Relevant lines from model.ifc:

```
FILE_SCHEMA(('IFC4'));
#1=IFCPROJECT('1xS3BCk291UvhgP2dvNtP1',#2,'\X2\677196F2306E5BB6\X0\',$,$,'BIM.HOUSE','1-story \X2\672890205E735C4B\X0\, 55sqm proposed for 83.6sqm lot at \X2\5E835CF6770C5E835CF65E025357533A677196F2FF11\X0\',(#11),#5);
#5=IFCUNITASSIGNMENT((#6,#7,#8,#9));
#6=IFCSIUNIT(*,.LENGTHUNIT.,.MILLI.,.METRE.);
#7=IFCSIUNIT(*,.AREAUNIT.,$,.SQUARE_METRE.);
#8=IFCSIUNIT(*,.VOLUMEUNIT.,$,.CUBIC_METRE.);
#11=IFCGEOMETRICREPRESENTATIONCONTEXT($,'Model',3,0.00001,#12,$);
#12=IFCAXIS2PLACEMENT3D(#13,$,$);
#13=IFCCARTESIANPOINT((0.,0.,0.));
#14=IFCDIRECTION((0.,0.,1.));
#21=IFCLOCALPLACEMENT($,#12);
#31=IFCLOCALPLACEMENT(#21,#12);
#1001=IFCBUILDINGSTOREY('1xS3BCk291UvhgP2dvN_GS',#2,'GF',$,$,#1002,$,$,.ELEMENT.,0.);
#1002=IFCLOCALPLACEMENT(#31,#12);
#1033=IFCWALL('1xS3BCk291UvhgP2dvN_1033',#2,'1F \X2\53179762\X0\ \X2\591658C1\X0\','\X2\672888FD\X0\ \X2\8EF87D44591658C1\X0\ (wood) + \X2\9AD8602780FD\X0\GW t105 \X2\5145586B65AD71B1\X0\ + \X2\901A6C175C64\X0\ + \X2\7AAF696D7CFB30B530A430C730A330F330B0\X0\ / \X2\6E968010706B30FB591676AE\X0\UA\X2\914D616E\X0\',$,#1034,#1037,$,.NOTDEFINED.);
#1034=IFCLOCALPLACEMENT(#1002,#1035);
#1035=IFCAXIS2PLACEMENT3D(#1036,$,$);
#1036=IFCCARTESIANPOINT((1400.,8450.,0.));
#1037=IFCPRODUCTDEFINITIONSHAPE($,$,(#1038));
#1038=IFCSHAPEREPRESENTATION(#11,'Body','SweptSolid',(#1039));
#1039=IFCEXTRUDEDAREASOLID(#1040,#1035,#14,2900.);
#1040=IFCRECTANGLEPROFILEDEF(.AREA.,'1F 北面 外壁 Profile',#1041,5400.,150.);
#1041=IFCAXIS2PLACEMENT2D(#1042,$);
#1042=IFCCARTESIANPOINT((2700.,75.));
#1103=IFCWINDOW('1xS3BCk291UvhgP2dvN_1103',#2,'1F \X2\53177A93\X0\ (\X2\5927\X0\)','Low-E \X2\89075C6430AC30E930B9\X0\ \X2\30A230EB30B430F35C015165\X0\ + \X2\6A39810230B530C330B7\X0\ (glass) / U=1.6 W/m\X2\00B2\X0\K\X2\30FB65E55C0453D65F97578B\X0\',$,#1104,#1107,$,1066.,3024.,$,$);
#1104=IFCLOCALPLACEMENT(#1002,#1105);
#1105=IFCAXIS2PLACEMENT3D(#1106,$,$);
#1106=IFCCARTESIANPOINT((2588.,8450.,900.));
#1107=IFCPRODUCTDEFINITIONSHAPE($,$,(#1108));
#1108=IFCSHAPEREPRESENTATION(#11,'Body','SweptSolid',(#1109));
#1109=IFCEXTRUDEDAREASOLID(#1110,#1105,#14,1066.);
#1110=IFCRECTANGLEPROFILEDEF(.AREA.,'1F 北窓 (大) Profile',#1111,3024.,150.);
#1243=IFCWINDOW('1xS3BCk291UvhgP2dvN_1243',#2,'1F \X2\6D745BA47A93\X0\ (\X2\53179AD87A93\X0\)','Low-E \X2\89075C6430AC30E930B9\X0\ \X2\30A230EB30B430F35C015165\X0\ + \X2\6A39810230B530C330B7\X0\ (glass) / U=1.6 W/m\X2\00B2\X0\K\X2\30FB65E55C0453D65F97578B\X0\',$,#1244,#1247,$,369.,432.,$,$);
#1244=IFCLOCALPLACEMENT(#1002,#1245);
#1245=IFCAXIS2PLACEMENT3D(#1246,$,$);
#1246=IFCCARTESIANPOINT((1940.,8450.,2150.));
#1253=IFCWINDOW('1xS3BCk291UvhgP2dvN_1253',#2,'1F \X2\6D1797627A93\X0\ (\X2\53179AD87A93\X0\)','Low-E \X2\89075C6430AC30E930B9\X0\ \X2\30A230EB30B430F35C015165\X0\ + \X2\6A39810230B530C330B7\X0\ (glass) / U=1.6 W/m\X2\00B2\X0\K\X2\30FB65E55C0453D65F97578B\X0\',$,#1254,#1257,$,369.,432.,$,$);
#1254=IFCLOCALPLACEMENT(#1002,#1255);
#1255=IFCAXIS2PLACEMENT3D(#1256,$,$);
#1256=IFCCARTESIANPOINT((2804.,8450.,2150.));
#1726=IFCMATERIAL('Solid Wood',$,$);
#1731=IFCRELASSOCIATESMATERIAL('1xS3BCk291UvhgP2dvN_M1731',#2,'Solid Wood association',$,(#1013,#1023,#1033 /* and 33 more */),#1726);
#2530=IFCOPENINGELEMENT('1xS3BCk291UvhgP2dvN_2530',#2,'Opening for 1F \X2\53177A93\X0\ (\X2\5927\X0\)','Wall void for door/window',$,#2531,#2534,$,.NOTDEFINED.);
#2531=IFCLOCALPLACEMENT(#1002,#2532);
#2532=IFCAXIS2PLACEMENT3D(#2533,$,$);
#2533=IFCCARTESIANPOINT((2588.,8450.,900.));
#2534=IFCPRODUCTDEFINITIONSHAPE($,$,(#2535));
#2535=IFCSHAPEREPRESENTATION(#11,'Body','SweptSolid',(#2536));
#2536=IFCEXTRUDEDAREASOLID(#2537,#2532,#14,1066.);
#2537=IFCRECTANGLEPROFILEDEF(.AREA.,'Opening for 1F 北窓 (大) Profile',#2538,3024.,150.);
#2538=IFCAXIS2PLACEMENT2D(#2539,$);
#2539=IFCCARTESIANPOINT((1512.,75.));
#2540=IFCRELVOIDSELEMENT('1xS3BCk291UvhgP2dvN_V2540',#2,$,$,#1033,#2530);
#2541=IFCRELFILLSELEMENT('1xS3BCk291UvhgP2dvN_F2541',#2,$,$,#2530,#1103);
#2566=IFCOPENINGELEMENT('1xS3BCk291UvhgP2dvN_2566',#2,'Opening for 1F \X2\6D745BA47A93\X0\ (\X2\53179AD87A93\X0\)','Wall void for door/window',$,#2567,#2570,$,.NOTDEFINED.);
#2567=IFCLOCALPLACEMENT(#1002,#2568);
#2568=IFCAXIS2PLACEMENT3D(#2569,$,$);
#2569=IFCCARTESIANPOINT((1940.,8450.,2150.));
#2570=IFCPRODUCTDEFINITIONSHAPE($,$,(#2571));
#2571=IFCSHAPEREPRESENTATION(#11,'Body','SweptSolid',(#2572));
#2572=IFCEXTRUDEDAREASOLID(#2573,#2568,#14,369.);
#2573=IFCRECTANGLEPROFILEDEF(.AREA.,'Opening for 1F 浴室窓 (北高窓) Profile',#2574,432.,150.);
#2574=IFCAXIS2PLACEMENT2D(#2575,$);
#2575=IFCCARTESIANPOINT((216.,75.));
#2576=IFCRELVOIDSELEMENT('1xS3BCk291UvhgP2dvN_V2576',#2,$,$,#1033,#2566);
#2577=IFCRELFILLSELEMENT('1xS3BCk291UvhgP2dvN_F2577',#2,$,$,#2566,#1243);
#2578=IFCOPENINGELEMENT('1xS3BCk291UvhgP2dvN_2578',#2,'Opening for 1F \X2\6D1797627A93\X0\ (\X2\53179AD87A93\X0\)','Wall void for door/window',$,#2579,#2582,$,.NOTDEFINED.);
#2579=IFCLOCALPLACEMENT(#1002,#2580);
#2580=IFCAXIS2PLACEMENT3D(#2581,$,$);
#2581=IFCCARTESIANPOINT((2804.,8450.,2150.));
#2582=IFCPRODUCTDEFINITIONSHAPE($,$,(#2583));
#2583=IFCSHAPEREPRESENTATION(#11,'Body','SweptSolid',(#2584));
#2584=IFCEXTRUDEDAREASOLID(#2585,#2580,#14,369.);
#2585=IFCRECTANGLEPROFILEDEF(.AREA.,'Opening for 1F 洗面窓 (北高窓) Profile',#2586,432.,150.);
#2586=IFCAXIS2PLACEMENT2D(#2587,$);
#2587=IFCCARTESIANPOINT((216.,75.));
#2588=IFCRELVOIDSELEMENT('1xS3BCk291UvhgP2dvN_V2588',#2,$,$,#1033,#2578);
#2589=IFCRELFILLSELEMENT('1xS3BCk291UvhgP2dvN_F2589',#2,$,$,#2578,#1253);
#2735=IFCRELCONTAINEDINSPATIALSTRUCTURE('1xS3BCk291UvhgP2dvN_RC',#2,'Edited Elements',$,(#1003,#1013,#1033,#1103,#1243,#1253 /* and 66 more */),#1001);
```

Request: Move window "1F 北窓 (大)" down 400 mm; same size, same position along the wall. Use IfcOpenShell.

```python
import numpy as np
import ifcopenshell
import ifcopenshell.api.geometry
import ifcopenshell.util.placement
import ifcopenshell.util.unit

model = ifcopenshell.open("model.ifc")
unit_scale = ifcopenshell.util.unit.calculate_unit_scale(model)

window = model.by_guid("1xS3BCk291UvhgP2dvN_1103")
opening = window.FillsVoids[0].RelatingOpeningElement
dz = -0.4 / unit_scale

shift = np.array([0.0, 0.0, dz])
# The window is not placed relative to its opening, so move both.
for product in (opening, window):
    matrix = ifcopenshell.util.placement.get_local_placement(product.ObjectPlacement)
    matrix[:3, 3] += shift
    ifcopenshell.api.geometry.edit_object_placement(model, product=product, matrix=matrix, is_si=False)

print(f"moved by {dz * unit_scale:+.3f} m")

model.write("model-out.ifc")
```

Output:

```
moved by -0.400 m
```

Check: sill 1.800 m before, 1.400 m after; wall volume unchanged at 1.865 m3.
